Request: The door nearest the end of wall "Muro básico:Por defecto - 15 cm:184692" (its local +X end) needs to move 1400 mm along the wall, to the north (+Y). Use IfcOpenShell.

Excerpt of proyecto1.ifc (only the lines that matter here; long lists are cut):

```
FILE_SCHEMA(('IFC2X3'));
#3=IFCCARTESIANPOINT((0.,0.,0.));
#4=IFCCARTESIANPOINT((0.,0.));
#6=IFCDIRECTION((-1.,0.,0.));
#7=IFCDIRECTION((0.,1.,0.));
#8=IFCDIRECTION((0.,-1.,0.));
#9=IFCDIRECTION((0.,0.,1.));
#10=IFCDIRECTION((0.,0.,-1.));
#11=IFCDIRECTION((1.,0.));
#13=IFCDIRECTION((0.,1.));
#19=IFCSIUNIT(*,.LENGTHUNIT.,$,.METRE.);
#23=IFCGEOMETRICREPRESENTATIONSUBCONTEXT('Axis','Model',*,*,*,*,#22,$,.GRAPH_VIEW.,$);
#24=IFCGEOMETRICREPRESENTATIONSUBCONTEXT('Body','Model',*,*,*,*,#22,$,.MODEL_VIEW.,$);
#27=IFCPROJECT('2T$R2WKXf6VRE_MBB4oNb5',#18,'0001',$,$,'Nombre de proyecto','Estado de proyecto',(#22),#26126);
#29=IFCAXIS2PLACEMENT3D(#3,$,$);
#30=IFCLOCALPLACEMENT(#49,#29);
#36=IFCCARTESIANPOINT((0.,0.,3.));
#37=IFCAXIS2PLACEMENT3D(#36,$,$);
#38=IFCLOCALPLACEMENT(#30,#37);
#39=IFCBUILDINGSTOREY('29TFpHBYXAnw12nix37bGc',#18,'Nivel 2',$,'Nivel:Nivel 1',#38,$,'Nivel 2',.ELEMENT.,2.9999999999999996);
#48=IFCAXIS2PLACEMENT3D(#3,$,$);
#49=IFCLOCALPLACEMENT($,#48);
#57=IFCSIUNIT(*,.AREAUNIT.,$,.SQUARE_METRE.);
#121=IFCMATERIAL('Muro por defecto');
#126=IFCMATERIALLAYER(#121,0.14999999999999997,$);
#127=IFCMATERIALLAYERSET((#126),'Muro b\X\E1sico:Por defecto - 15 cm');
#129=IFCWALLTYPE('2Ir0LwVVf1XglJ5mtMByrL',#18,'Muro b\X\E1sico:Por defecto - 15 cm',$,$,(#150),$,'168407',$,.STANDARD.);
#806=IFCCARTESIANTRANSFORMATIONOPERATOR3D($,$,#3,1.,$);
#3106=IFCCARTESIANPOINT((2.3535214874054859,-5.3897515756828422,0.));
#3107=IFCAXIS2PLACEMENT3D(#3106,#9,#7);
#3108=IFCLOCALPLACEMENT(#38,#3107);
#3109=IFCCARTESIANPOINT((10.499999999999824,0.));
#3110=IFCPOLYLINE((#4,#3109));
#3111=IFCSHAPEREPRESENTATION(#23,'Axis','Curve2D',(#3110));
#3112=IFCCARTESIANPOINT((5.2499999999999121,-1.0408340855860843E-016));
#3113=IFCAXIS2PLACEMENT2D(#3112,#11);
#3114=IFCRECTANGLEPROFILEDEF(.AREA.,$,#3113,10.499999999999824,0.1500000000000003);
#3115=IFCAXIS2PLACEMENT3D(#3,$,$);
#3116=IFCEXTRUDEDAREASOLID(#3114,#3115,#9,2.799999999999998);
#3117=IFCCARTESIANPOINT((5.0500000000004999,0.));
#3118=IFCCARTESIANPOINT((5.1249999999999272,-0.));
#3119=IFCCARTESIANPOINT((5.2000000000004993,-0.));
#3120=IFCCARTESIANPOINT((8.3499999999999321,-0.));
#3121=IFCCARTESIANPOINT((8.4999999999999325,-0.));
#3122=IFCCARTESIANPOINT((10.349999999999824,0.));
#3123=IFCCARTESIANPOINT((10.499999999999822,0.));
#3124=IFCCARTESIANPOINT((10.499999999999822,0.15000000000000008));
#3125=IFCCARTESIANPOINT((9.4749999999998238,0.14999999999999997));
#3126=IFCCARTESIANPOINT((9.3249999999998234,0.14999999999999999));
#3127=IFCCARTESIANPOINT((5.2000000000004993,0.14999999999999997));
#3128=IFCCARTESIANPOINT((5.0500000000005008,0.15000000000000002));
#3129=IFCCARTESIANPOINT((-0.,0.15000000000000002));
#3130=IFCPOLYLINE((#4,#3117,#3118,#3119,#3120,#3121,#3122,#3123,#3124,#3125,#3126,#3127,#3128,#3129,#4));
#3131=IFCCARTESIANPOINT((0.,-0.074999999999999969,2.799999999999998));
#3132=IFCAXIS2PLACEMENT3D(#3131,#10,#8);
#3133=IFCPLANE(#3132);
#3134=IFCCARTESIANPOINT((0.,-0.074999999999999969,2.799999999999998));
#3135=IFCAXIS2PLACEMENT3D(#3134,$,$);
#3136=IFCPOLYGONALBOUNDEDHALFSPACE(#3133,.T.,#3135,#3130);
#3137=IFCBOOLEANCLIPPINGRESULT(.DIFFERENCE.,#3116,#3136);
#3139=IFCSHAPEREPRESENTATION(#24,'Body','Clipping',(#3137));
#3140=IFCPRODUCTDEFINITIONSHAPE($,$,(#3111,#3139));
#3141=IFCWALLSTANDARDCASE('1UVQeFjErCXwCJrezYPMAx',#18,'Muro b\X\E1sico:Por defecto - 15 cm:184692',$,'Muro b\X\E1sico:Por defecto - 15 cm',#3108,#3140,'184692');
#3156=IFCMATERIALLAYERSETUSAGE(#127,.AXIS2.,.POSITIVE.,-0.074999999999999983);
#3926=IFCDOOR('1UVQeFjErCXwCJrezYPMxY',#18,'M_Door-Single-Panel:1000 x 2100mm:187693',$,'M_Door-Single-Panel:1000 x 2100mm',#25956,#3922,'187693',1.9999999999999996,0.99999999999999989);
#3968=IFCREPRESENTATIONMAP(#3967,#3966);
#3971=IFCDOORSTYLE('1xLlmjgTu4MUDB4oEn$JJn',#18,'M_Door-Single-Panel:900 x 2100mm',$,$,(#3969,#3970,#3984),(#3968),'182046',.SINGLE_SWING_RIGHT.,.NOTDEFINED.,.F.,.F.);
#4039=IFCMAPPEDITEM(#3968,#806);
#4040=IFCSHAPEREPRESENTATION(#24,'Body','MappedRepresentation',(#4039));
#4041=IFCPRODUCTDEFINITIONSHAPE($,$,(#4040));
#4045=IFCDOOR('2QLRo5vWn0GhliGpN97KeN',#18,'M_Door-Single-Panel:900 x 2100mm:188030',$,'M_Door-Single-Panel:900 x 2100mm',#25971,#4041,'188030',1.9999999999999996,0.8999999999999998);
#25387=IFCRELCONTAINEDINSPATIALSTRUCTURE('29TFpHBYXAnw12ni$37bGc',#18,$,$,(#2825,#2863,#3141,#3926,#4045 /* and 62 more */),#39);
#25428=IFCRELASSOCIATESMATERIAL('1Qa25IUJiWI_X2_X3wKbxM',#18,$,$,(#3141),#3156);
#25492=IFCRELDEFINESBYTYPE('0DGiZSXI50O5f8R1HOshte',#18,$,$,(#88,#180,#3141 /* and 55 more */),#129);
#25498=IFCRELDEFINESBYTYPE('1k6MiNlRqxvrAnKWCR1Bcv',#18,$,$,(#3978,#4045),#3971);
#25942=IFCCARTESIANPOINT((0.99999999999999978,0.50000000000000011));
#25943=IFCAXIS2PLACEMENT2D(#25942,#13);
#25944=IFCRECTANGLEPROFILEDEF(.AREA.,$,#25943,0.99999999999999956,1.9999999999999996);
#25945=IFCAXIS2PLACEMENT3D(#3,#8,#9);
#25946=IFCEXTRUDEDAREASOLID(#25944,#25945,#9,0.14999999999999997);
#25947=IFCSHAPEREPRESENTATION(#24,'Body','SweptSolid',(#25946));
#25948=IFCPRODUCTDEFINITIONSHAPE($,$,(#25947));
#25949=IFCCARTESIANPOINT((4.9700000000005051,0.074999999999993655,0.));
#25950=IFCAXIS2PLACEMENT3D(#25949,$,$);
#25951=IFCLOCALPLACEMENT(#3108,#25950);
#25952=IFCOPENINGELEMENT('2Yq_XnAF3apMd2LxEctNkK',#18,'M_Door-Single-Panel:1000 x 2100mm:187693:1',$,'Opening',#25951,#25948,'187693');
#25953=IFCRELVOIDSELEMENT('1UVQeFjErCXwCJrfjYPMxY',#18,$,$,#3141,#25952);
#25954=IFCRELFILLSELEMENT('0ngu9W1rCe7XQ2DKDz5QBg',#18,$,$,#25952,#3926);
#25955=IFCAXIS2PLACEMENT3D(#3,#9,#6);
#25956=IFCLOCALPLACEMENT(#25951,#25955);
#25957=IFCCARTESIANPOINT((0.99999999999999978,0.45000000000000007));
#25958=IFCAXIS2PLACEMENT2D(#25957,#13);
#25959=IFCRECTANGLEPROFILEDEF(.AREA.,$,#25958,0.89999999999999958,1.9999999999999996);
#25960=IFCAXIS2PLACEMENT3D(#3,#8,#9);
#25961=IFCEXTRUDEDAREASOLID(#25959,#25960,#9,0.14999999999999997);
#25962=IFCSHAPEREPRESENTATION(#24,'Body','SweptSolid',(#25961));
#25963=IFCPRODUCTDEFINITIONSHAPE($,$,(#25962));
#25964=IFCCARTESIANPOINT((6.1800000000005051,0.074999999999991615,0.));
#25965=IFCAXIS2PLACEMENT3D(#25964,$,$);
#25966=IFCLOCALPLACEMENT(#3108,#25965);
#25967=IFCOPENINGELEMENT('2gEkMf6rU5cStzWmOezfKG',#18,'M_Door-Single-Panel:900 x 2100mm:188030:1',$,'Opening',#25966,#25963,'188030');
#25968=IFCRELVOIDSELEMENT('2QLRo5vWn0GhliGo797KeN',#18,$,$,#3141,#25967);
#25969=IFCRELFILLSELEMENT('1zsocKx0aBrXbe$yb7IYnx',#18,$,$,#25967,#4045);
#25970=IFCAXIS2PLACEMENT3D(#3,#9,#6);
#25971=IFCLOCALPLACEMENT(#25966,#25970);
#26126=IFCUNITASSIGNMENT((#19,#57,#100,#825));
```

```python
import ifcopenshell
import ifcopenshell.api.geometry
import ifcopenshell.util.placement
import ifcopenshell.util.unit

model = ifcopenshell.open("proyecto1.ifc")
unit_scale = ifcopenshell.util.unit.calculate_unit_scale(model)

door = model.by_id(4045)
opening = door.FillsVoids[0].RelatingOpeningElement
wall = opening.VoidsElements[0].RelatingBuildingElement

wall_matrix = ifcopenshell.util.placement.get_local_placement(wall.ObjectPlacement)
shift = wall_matrix[:3, 0] * 1.4 / unit_scale
before = ifcopenshell.util.placement.get_local_placement(door.ObjectPlacement)[:3, 3].copy()

# The door is placed relative to its opening, so it follows when the opening moves.
matrix = ifcopenshell.util.placement.get_local_placement(opening.ObjectPlacement)
matrix[:3, 3] += shift
ifcopenshell.api.geometry.edit_object_placement(
    model, product=opening, matrix=matrix, is_si=False, should_transform_children=True
)

after = ifcopenshell.util.placement.get_local_placement(door.ObjectPlacement)[:3, 3]
print("door moved by", (after - before).round(3) + 0.0)

model.write("proyecto1_rev.ifc")
```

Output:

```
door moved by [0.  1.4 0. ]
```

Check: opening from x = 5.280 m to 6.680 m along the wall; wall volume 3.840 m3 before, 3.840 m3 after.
